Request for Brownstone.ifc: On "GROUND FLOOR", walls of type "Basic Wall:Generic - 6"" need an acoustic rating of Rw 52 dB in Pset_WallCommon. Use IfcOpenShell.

First a look at what the model holds.

```python
import ifcopenshell
import ifcopenshell.util.element

model = ifcopenshell.open("Brownstone.ifc")
print(model.schema)
storey = next(s for s in model.by_type("IfcBuildingStorey") if s.Name == "GROUND FLOOR")
walls = [e for e in ifcopenshell.util.element.get_decomposition(storey) if e.is_a("IfcWall")]
seen = {}
for e in walls:
    element_type = ifcopenshell.util.element.get_type(e)
    key = (element_type.Name if element_type != e and element_type else None, ifcopenshell.util.element.get_pset(e, "Pset_WallCommon", "AcousticRating"))
    seen[key] = seen.get(key, 0) + 1
for (name, value), count in sorted(seen.items(), key=str):
    print(count, "x", name, "|", value)
```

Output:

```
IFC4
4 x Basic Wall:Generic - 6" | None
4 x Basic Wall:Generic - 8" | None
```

```python
import ifcopenshell
import ifcopenshell.api.pset
import ifcopenshell.util.element

model = ifcopenshell.open("Brownstone.ifc")

storey = next(s for s in model.by_type("IfcBuildingStorey") if s.Name == "GROUND FLOOR")
walls = [e for e in ifcopenshell.util.element.get_decomposition(storey) if e.is_a("IfcWall")]

count = 0
for e in walls:
    element_type = ifcopenshell.util.element.get_type(e)
    if element_type in (None, e) or element_type.Name != 'Basic Wall:Generic - 6"':
        continue
    # add_pset returns the element's existing set when there is one.
    pset = ifcopenshell.api.pset.add_pset(model, product=e, name="Pset_WallCommon")
    ifcopenshell.api.pset.edit_pset(model, pset=pset, properties={"AcousticRating": "Rw 52 dB"})
    count += 1

print(count, "walls updated")

model.write("Brownstone_edited.ifc")
```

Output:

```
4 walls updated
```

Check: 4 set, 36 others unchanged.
